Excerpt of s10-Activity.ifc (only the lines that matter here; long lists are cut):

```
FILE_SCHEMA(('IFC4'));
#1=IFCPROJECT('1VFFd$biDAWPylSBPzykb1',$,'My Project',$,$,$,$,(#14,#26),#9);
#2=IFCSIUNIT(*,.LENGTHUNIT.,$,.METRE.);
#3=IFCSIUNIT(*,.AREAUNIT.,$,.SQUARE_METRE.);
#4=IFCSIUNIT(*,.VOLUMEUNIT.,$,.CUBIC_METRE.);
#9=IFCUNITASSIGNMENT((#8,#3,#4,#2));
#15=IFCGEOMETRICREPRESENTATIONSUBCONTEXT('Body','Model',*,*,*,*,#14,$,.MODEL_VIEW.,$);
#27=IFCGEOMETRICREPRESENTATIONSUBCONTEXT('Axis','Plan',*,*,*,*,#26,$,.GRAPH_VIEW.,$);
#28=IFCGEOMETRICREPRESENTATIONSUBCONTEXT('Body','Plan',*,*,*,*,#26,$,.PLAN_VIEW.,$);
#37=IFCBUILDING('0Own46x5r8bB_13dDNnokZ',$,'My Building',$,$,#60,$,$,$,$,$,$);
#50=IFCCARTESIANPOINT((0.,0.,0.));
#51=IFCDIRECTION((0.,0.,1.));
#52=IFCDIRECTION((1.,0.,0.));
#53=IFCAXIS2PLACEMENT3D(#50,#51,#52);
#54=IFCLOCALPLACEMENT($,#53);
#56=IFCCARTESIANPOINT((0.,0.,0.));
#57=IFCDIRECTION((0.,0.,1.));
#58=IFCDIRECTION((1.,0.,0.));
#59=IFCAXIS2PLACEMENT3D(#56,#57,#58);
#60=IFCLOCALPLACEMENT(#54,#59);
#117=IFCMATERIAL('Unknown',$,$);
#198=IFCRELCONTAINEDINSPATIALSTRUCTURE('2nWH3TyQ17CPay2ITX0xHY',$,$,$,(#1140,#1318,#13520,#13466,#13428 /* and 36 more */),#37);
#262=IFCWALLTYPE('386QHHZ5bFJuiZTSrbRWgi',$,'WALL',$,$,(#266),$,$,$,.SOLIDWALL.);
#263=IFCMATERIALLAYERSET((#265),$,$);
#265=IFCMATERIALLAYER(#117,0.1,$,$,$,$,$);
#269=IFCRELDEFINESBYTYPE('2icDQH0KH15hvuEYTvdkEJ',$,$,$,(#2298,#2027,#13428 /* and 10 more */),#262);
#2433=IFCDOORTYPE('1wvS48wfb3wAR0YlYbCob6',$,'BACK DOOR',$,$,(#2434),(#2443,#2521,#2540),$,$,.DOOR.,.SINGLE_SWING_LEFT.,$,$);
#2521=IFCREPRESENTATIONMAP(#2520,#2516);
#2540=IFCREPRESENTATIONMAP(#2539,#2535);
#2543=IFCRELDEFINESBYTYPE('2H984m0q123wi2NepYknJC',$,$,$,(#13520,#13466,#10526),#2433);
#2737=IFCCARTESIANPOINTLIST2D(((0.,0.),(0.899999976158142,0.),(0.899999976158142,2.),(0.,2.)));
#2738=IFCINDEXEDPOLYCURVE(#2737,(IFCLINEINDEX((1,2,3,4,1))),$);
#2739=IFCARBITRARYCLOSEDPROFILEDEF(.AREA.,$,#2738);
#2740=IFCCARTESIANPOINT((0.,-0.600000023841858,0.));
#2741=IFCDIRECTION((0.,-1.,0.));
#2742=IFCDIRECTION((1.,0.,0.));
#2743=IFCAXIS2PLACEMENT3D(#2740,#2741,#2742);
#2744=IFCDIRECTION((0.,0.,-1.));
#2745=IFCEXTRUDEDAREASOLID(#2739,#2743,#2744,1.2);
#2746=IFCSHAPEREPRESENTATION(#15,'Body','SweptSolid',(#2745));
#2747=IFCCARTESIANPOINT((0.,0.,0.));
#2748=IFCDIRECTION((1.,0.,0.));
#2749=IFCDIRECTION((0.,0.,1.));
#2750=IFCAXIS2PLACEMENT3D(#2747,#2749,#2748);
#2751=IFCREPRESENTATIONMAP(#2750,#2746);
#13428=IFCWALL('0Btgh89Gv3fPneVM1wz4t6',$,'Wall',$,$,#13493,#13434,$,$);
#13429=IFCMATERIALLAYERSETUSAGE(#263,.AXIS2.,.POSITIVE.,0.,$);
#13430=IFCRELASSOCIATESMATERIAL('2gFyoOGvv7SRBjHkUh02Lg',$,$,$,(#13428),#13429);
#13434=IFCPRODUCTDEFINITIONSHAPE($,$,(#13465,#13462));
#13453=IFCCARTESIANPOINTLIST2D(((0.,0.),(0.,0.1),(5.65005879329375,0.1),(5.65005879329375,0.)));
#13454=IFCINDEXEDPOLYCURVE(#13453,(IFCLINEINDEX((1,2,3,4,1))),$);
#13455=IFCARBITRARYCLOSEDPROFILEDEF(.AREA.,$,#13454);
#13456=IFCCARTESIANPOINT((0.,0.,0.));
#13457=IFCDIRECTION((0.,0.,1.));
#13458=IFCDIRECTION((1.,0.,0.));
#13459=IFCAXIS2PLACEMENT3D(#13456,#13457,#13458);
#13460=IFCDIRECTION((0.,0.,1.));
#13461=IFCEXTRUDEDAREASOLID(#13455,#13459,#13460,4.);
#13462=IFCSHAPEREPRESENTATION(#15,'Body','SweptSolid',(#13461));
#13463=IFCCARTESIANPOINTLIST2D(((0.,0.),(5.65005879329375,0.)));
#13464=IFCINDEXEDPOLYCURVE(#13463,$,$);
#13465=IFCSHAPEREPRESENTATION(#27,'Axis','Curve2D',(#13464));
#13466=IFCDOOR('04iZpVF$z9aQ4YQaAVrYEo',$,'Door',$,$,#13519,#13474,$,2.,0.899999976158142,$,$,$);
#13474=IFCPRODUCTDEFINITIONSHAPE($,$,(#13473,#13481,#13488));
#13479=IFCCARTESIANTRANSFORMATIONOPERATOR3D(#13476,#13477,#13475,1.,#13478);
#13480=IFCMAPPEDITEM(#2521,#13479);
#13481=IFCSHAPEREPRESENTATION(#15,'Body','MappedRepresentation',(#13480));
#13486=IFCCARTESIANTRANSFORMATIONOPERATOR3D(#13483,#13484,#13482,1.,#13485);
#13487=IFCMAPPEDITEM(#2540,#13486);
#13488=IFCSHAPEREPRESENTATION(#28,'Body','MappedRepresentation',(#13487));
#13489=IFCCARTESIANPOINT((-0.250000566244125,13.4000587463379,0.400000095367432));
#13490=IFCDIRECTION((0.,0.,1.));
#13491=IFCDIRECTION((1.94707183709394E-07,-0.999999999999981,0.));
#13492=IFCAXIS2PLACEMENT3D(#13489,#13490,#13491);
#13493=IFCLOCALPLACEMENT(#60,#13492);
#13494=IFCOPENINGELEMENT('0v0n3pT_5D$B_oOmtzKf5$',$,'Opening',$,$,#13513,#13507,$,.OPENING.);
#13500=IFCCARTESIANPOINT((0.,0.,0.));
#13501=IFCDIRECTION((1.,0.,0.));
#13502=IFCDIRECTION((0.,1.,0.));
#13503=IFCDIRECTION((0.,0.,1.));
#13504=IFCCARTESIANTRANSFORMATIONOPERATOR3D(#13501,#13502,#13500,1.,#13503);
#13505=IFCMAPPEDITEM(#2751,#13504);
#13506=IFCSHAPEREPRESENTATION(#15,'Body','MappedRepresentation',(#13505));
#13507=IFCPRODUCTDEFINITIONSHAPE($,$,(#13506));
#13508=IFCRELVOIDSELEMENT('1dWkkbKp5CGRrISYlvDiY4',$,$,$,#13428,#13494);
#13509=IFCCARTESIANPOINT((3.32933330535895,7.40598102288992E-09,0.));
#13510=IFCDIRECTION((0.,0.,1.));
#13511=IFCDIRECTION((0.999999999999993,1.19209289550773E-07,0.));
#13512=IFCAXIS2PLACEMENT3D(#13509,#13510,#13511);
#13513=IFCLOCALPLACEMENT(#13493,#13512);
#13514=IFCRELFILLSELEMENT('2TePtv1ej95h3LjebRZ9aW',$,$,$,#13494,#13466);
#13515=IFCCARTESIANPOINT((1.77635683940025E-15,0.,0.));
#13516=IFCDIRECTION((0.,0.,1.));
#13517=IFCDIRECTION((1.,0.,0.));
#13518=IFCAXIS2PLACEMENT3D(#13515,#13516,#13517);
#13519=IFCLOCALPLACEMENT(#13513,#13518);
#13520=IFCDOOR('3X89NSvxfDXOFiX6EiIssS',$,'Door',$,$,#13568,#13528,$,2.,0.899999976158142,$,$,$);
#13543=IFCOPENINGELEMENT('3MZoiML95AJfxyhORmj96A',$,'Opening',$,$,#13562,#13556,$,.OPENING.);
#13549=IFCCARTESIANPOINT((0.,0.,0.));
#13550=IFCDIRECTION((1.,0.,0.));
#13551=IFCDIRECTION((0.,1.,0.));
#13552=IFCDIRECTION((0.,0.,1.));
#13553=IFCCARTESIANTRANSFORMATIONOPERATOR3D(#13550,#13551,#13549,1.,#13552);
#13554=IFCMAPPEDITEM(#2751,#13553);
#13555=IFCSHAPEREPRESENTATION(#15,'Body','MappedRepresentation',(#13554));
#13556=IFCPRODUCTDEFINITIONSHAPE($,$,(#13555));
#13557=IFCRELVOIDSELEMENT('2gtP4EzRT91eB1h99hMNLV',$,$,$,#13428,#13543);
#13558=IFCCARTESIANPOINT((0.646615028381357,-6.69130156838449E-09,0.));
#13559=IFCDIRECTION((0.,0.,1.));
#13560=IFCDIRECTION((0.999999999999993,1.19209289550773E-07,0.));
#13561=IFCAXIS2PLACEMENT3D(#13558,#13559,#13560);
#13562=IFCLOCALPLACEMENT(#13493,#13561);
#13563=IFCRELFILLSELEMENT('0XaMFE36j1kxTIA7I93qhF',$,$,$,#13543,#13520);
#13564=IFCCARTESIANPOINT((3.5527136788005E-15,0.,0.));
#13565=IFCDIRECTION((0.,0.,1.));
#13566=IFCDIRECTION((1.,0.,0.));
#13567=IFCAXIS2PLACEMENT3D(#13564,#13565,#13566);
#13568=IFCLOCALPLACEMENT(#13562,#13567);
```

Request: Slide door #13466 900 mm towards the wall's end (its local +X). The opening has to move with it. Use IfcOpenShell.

```python
import ifcopenshell
import ifcopenshell.api.geometry
import ifcopenshell.util.placement

model = ifcopenshell.open("s10-Activity.ifc")

door = model.by_guid("04iZpVF$z9aQ4YQaAVrYEo")
opening = door.FillsVoids[0].RelatingOpeningElement
wall = opening.VoidsElements[0].RelatingBuildingElement

wall_matrix = ifcopenshell.util.placement.get_local_placement(wall.ObjectPlacement)
shift = wall_matrix[:3, 0] * 0.9
before = ifcopenshell.util.placement.get_local_placement(door.ObjectPlacement)[:3, 3].copy()

# The door is placed relative to its opening, so it follows when the opening moves.
matrix = ifcopenshell.util.placement.get_local_placement(opening.ObjectPlacement)
matrix[:3, 3] += shift
ifcopenshell.api.geometry.edit_object_placement(
    model, product=opening, matrix=matrix, is_si=False, should_transform_children=True
)

after = ifcopenshell.util.placement.get_local_placement(door.ObjectPlacement)[:3, 3]
print("door moved by", (after - before).round(3) + 0.0)

model.write("s10-Activity-out.ifc")
```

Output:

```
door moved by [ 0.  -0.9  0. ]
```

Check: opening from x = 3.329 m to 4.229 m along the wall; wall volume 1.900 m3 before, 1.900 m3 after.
